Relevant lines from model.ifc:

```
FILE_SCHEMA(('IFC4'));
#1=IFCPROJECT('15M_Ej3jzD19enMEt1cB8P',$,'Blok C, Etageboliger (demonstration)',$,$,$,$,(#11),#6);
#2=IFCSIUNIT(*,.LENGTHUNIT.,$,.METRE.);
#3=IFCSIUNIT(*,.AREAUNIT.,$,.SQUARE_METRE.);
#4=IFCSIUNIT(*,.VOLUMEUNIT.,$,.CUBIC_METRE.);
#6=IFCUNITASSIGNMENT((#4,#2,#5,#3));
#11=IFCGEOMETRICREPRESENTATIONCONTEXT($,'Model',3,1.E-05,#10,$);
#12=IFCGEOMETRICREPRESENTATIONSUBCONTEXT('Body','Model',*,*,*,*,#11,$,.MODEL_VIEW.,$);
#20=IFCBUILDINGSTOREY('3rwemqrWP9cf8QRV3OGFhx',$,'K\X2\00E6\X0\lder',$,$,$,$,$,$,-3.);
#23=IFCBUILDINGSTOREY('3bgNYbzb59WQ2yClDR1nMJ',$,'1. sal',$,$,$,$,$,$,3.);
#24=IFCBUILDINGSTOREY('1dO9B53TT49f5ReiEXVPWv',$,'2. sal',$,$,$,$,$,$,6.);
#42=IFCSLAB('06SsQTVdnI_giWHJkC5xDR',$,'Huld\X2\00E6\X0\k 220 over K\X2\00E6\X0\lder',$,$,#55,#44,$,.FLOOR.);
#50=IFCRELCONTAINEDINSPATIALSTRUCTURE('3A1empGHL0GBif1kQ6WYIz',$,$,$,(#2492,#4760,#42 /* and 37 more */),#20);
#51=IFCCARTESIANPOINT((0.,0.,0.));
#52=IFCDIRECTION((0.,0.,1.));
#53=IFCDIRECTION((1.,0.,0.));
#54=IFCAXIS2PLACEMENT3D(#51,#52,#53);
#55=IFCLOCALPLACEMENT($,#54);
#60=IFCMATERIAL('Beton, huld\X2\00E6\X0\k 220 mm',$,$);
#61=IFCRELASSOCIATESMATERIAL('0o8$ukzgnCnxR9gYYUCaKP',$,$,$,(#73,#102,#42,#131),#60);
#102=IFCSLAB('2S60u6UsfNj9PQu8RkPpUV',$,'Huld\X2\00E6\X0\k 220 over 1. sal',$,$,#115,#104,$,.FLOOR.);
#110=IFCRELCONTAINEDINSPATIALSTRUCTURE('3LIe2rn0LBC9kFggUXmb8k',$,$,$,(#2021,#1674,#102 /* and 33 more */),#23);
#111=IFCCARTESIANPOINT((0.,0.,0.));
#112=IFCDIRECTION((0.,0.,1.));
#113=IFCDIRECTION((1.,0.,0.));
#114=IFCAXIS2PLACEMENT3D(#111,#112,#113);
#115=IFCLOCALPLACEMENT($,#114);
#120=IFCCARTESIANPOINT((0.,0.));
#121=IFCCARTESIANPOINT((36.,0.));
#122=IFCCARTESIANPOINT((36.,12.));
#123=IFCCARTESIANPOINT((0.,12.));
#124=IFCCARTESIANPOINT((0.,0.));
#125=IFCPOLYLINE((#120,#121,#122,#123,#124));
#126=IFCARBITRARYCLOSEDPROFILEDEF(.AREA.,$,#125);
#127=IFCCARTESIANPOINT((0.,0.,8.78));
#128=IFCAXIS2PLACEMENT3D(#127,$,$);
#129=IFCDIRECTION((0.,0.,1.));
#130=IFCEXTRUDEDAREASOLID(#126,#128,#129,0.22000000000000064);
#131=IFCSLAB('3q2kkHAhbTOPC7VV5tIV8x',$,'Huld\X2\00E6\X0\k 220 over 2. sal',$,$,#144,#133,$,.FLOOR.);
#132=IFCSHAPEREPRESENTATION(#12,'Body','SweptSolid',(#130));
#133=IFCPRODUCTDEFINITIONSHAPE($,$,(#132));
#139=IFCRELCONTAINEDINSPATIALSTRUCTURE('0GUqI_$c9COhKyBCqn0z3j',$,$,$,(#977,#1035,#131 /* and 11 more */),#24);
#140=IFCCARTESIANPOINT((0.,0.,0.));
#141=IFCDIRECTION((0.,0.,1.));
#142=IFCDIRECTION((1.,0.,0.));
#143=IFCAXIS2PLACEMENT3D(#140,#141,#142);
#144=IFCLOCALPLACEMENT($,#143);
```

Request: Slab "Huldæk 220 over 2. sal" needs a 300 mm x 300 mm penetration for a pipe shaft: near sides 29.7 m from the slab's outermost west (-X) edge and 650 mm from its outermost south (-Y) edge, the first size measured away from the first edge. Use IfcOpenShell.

```python
import numpy as np
import ifcopenshell
import ifcopenshell.api.feature
import ifcopenshell.api.geometry
import ifcopenshell.api.root
import ifcopenshell.geom
import ifcopenshell.util.placement
import ifcopenshell.util.representation
import ifcopenshell.util.shape
import ifcopenshell.util.unit

model = ifcopenshell.open("model.ifc")
unit_scale = ifcopenshell.util.unit.calculate_unit_scale(model)
settings = ifcopenshell.geom.settings()


def volume(element):
    """Net volume in cubic metres, openings subtracted."""
    shape = ifcopenshell.geom.create_shape(settings, element)
    return ifcopenshell.util.shape.get_volume(shape.geometry)


slab = model.by_guid("3q2kkHAhbTOPC7VV5tIV8x")
before = volume(slab)

# Extent in the slab's own axes, in metres. The edges named are its -X and -Y sides.
slab_shape = ifcopenshell.geom.create_shape(settings, slab)
vertices = ifcopenshell.util.shape.get_vertices(slab_shape.geometry)
x_min, y_min, bottom = vertices.min(axis=0)
top = vertices[:, 2].max()

opening = ifcopenshell.api.root.create_entity(model, ifc_class="IfcOpeningElement", name="Pipe shaft opening", predefined_type="OPENING")
context = ifcopenshell.util.representation.get_context(model, "Model", "Body", "MODEL_VIEW")
width, depth = 0.3, 0.3
outline = [(0.0, 0.0), (width, 0.0), (width, depth), (0.0, depth), (0.0, 0.0)]
# Overshoot both faces by 50 mm so the cut is clean.
shape = ifcopenshell.api.geometry.add_slab_representation(
    model, context=context, depth=top - bottom + 0.1, polyline=outline
)
ifcopenshell.api.geometry.assign_representation(model, product=opening, representation=shape)

matrix = ifcopenshell.util.placement.get_local_placement(slab.ObjectPlacement)
matrix[:, 3] = matrix @ np.append(np.array([x_min + 29.7, y_min + 0.65, bottom - 0.05]) / unit_scale, 1.0)
ifcopenshell.api.geometry.edit_object_placement(model, product=opening, matrix=matrix, is_si=False)
ifcopenshell.api.feature.add_feature(model, feature=opening, element=slab)

after = volume(slab)

print(f"slab volume {before:.3f} -> {after:.3f} m3")

model.write("model_rev.ifc")
```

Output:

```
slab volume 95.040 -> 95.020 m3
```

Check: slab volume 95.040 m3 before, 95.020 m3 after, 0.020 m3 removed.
